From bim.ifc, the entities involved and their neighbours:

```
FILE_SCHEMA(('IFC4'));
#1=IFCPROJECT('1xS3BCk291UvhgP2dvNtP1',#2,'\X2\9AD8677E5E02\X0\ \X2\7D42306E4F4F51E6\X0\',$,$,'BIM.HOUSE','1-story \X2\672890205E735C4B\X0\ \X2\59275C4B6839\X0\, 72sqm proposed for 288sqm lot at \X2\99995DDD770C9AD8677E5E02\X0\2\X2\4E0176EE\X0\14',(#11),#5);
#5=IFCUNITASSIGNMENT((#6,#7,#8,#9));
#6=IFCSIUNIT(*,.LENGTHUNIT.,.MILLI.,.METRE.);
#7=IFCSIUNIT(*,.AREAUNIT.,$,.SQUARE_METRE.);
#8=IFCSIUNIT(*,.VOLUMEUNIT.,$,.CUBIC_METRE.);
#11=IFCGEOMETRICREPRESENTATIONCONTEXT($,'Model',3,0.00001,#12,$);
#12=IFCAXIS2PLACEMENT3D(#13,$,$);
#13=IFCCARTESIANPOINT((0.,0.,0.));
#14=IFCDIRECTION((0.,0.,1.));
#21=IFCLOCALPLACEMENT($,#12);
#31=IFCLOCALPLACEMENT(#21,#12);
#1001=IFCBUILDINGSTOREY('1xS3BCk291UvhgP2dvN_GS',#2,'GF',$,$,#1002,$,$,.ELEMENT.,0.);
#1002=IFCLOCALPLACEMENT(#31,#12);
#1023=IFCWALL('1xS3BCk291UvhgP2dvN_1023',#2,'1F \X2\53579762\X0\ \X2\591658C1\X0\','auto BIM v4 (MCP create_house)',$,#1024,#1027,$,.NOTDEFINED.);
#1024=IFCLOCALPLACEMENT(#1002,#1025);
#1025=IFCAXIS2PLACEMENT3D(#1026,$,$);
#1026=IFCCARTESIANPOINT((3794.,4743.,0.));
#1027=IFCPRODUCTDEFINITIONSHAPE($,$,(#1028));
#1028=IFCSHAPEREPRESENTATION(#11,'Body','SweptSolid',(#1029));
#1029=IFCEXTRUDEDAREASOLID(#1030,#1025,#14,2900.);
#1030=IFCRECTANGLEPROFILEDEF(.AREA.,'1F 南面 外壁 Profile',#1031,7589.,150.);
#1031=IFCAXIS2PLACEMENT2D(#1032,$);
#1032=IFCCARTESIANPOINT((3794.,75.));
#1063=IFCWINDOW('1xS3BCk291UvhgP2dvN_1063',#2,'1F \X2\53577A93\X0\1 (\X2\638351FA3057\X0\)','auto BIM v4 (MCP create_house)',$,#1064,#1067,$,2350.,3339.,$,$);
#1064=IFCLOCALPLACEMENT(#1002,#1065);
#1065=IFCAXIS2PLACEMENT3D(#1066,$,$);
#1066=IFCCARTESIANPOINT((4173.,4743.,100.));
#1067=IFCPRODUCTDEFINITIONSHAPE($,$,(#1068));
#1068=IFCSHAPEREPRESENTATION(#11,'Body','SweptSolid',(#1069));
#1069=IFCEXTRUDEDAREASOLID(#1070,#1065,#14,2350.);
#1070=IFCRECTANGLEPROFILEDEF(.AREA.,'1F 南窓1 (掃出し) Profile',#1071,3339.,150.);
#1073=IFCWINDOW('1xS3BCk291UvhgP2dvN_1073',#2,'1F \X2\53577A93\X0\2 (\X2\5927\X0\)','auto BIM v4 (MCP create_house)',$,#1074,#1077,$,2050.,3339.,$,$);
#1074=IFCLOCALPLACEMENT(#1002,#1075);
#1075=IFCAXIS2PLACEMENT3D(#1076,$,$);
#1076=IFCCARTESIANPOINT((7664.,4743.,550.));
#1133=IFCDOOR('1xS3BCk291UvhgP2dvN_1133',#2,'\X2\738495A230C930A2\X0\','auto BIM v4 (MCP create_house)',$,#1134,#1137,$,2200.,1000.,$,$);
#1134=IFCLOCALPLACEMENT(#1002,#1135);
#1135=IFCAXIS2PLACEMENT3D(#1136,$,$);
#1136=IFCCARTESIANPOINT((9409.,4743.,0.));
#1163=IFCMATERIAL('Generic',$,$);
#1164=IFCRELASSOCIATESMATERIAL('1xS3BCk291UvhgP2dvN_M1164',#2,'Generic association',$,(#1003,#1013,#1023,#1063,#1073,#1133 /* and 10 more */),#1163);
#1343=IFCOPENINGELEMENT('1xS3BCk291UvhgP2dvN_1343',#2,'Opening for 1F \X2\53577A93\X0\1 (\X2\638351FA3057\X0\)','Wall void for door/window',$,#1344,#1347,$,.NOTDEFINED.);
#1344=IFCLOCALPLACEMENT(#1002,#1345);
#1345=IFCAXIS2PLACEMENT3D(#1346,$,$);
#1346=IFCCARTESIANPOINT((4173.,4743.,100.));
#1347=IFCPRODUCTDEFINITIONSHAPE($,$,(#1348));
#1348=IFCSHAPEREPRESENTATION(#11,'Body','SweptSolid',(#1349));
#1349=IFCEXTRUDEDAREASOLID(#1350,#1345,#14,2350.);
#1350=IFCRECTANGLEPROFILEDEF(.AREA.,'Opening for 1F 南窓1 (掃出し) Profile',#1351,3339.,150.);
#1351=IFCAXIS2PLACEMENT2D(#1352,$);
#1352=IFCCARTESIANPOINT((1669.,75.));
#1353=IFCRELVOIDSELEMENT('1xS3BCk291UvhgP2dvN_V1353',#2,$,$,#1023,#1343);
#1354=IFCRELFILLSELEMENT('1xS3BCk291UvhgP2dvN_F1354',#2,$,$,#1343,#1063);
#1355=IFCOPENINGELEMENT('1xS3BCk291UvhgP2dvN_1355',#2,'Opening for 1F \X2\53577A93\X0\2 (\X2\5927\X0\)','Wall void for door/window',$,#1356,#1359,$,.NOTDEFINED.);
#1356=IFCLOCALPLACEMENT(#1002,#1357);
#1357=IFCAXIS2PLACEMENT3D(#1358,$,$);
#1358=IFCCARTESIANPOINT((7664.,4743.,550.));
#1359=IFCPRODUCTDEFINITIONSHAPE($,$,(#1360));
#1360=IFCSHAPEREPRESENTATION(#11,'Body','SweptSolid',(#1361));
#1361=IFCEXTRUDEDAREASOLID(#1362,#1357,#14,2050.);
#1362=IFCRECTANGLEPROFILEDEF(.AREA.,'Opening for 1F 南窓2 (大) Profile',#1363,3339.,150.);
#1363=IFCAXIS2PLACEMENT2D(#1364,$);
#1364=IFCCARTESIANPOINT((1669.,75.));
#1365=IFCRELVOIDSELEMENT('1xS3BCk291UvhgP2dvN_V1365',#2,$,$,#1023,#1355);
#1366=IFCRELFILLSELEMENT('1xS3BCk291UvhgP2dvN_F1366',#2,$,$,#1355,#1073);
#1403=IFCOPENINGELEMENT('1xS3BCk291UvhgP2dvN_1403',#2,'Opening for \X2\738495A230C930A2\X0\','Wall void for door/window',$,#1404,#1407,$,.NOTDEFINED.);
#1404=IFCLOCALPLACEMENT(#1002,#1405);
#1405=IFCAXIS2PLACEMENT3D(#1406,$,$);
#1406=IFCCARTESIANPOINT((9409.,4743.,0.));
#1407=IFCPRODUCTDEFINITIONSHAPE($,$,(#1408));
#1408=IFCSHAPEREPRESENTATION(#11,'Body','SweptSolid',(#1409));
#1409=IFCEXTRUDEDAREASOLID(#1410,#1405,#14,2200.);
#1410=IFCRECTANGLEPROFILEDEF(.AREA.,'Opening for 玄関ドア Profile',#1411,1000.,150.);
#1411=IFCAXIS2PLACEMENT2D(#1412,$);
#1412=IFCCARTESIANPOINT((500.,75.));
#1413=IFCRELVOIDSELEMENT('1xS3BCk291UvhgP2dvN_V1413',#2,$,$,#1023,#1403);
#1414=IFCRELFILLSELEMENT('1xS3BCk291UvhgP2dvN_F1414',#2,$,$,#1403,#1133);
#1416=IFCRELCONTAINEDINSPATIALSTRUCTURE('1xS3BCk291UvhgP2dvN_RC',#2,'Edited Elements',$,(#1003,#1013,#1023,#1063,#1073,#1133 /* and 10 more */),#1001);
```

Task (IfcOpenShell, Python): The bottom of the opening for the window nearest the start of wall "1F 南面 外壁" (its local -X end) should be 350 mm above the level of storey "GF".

```python
import numpy as np
import ifcopenshell
import ifcopenshell.api.geometry
import ifcopenshell.geom
import ifcopenshell.util.element
import ifcopenshell.util.placement
import ifcopenshell.util.shape
import ifcopenshell.util.unit

model = ifcopenshell.open("bim.ifc")
unit_scale = ifcopenshell.util.unit.calculate_unit_scale(model)

window = model.by_id(1063)
opening = window.FillsVoids[0].RelatingOpeningElement
storey = ifcopenshell.util.element.get_container(window, ifc_class="IfcBuildingStorey")
level = ifcopenshell.util.placement.get_local_placement(storey.ObjectPlacement)[2, 3]

# The opening's origin need not be at the sill, so measure its lowest point.
shape = ifcopenshell.geom.create_shape(ifcopenshell.geom.settings(), opening)
bottom = ifcopenshell.util.shape.get_shape_bottom_elevation(shape, shape.geometry) / unit_scale
dz = level + 0.35 / unit_scale - bottom

shift = np.array([0.0, 0.0, dz])
# The window is not placed relative to its opening, so move both.
for product in (opening, window):
    matrix = ifcopenshell.util.placement.get_local_placement(product.ObjectPlacement)
    matrix[:3, 3] += shift
    ifcopenshell.api.geometry.edit_object_placement(model, product=product, matrix=matrix, is_si=False)

print(f"moved by {dz * unit_scale:+.3f} m")

model.write("bim_rev.ifc")
```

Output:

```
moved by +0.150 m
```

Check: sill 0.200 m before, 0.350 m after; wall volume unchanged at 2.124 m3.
